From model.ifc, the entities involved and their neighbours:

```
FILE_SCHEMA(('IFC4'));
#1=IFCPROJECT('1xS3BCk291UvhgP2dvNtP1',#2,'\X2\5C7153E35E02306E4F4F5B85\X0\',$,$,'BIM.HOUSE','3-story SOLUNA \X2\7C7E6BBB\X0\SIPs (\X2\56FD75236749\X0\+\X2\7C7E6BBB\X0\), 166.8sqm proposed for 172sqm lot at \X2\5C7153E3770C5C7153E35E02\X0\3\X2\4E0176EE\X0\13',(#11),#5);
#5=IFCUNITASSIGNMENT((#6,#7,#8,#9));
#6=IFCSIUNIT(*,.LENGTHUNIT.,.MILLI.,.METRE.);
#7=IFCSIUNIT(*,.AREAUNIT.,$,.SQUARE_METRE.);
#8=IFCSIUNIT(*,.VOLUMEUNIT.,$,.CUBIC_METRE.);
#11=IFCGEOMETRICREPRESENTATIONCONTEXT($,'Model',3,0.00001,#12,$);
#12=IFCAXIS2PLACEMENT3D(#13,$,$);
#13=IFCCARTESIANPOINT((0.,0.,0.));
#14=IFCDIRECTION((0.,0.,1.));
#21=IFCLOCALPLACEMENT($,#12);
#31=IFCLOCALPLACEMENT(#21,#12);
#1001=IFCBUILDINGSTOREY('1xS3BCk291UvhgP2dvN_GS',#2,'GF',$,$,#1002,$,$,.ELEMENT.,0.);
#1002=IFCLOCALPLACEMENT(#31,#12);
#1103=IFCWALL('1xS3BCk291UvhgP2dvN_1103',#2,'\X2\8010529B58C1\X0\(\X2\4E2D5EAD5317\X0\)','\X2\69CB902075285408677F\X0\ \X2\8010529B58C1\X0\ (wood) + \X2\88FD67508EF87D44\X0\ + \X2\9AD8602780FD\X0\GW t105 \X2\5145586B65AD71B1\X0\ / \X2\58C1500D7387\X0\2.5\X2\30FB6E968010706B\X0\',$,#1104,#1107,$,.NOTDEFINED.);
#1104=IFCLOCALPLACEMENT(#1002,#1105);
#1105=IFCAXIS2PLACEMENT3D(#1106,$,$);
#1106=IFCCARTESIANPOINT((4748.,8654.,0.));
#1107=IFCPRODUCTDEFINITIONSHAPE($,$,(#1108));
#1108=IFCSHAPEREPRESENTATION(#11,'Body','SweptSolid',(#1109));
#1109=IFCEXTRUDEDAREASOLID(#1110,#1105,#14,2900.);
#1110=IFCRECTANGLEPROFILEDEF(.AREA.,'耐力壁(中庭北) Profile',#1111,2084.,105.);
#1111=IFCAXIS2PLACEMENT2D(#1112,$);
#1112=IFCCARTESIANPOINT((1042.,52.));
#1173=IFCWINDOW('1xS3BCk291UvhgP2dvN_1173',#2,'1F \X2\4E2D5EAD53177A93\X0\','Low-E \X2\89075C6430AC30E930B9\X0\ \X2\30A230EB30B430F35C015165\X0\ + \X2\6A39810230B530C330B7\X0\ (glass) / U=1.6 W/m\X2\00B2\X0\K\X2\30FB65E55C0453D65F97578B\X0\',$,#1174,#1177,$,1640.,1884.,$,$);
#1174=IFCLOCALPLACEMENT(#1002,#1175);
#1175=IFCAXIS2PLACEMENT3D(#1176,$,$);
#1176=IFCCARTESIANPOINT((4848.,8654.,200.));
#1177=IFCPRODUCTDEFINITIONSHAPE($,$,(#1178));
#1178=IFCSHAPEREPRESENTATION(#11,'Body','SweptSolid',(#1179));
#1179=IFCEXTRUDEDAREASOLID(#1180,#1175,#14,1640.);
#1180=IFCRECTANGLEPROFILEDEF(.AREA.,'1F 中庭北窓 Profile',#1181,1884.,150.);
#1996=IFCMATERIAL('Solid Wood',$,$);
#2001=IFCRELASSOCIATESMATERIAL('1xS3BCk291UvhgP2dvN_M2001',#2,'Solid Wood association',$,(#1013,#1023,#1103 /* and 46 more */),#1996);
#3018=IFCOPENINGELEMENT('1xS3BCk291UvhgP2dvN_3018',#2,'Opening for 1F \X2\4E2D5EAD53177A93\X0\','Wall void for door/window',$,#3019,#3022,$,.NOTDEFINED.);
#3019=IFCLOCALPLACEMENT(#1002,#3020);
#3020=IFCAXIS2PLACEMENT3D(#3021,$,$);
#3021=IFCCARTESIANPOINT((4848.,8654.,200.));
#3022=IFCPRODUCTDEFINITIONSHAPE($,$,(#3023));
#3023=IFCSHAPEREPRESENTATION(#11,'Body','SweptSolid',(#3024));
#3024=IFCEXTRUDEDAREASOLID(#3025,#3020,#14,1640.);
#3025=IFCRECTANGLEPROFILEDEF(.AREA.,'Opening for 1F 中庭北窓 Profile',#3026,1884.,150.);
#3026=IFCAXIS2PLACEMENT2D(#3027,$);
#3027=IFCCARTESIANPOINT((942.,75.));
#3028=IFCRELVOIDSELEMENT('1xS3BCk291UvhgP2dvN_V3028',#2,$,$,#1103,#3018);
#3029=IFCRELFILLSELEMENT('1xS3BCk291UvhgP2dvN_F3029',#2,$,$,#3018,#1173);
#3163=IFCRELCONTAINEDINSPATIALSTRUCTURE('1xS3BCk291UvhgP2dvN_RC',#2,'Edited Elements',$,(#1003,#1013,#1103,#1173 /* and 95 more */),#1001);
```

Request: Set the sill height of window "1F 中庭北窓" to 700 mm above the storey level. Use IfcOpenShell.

```python
import numpy as np
import ifcopenshell
import ifcopenshell.api.geometry
import ifcopenshell.geom
import ifcopenshell.util.element
import ifcopenshell.util.placement
import ifcopenshell.util.shape
import ifcopenshell.util.unit

model = ifcopenshell.open("model.ifc")
unit_scale = ifcopenshell.util.unit.calculate_unit_scale(model)

window = model.by_guid("1xS3BCk291UvhgP2dvN_1173")
opening = window.FillsVoids[0].RelatingOpeningElement
storey = ifcopenshell.util.element.get_container(window, ifc_class="IfcBuildingStorey")
level = ifcopenshell.util.placement.get_local_placement(storey.ObjectPlacement)[2, 3]

# The opening's origin need not be at the sill, so measure its lowest point.
shape = ifcopenshell.geom.create_shape(ifcopenshell.geom.settings(), opening)
bottom = ifcopenshell.util.shape.get_shape_bottom_elevation(shape, shape.geometry) / unit_scale
dz = level + 700.0 - bottom

shift = np.array([0.0, 0.0, dz])
# The window is not placed relative to its opening, so move both.
for product in (opening, window):
    matrix = ifcopenshell.util.placement.get_local_placement(product.ObjectPlacement)
    matrix[:3, 3] += shift
    ifcopenshell.api.geometry.edit_object_placement(model, product=product, matrix=matrix, is_si=False)

print(f"moved by {dz * unit_scale:+.3f} m")

model.write("model_edited.ifc")
```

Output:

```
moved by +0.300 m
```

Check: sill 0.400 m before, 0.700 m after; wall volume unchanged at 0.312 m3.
